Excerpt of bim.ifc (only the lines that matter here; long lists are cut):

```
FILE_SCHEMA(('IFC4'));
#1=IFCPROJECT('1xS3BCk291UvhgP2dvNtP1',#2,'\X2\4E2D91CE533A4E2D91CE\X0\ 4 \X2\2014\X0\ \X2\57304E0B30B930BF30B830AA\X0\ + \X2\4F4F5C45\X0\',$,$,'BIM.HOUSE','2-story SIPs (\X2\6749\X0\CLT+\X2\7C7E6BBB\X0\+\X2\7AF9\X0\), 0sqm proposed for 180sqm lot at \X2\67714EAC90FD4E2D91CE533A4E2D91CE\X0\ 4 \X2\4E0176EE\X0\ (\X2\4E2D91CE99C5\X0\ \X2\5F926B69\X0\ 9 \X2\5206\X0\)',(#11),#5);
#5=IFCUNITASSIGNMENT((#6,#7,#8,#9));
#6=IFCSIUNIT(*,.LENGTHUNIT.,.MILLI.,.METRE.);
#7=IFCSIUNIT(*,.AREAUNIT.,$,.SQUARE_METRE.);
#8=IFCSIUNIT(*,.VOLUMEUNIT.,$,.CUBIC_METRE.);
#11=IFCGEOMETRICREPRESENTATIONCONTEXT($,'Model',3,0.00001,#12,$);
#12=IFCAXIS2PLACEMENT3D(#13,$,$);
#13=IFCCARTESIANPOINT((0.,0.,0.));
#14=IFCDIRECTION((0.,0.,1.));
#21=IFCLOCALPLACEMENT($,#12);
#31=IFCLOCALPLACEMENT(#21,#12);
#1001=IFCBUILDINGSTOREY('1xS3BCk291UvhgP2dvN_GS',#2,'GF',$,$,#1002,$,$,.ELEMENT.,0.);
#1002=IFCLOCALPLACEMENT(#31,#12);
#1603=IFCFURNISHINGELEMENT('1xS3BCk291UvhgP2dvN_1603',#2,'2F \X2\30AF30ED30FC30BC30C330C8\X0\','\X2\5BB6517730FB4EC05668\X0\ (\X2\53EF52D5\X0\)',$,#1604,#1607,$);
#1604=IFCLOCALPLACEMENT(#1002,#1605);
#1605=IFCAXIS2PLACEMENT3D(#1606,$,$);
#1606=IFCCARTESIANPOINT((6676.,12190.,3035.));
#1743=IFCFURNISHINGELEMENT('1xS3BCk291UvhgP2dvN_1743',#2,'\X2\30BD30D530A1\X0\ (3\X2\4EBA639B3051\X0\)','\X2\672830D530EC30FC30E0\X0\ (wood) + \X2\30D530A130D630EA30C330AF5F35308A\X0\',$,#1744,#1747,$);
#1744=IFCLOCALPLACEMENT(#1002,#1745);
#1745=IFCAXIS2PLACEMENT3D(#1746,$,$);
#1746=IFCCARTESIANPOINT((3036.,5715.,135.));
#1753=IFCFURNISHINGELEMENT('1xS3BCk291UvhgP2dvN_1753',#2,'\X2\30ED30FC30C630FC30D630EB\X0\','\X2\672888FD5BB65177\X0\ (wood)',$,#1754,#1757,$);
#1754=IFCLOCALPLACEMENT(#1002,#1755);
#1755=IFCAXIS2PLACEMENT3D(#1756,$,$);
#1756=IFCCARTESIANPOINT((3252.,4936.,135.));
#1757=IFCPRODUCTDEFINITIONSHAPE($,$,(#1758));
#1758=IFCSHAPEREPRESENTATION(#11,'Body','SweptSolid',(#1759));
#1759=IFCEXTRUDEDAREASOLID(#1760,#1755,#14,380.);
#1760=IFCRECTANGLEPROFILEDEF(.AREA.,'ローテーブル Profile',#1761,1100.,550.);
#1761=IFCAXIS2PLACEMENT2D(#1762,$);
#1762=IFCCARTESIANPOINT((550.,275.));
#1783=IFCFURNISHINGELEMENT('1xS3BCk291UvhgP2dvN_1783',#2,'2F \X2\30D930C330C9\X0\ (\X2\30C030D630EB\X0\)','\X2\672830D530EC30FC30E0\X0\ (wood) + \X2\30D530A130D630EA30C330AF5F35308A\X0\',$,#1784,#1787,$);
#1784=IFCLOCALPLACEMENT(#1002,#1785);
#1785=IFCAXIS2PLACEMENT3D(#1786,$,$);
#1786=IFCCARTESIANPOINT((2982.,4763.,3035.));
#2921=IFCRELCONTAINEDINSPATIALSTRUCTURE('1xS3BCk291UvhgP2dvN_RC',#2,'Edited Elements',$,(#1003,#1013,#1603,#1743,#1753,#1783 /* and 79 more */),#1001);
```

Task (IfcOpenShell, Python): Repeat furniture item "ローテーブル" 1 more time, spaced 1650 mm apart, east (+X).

```python
import numpy as np
import ifcopenshell
import ifcopenshell.api.geometry
import ifcopenshell.api.root
import ifcopenshell.util.element
import ifcopenshell.util.placement

model = ifcopenshell.open("bim.ifc")


def reuse_history(source, copy):
    """copy_class also copies each property set's owner history, people and application; keep the originals."""
    for rel in copy.IsDefinedBy:
        if rel.is_a("IfcRelDefinesByProperties") and (history := rel.RelatingPropertyDefinition.OwnerHistory):
            rel.RelatingPropertyDefinition.OwnerHistory = source.OwnerHistory
            ifcopenshell.util.element.remove_deep2(model, history)


source = model.by_guid("1xS3BCk291UvhgP2dvN_1753")
base = ifcopenshell.util.placement.get_local_placement(source.ObjectPlacement)
step = np.array([1.0, 0.0, 0.0]) * 1650.0

for i in range(1, 2):
    copy = ifcopenshell.api.root.copy_class(model, product=source)
    copy.Representation = ifcopenshell.util.element.copy_deep(
        model, source.Representation, exclude=["IfcGeometricRepresentationContext", "IfcRepresentationMap"]
    )
    reuse_history(source, copy)
    matrix = base.copy()
    matrix[:3, 3] += i * step
    print("added at", matrix[:3, 3].round(3) + 0.0)
    ifcopenshell.api.geometry.edit_object_placement(model, product=copy, matrix=matrix, is_si=False)

model.write("bim_edited.ifc")
```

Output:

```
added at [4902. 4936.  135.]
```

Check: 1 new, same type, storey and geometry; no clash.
